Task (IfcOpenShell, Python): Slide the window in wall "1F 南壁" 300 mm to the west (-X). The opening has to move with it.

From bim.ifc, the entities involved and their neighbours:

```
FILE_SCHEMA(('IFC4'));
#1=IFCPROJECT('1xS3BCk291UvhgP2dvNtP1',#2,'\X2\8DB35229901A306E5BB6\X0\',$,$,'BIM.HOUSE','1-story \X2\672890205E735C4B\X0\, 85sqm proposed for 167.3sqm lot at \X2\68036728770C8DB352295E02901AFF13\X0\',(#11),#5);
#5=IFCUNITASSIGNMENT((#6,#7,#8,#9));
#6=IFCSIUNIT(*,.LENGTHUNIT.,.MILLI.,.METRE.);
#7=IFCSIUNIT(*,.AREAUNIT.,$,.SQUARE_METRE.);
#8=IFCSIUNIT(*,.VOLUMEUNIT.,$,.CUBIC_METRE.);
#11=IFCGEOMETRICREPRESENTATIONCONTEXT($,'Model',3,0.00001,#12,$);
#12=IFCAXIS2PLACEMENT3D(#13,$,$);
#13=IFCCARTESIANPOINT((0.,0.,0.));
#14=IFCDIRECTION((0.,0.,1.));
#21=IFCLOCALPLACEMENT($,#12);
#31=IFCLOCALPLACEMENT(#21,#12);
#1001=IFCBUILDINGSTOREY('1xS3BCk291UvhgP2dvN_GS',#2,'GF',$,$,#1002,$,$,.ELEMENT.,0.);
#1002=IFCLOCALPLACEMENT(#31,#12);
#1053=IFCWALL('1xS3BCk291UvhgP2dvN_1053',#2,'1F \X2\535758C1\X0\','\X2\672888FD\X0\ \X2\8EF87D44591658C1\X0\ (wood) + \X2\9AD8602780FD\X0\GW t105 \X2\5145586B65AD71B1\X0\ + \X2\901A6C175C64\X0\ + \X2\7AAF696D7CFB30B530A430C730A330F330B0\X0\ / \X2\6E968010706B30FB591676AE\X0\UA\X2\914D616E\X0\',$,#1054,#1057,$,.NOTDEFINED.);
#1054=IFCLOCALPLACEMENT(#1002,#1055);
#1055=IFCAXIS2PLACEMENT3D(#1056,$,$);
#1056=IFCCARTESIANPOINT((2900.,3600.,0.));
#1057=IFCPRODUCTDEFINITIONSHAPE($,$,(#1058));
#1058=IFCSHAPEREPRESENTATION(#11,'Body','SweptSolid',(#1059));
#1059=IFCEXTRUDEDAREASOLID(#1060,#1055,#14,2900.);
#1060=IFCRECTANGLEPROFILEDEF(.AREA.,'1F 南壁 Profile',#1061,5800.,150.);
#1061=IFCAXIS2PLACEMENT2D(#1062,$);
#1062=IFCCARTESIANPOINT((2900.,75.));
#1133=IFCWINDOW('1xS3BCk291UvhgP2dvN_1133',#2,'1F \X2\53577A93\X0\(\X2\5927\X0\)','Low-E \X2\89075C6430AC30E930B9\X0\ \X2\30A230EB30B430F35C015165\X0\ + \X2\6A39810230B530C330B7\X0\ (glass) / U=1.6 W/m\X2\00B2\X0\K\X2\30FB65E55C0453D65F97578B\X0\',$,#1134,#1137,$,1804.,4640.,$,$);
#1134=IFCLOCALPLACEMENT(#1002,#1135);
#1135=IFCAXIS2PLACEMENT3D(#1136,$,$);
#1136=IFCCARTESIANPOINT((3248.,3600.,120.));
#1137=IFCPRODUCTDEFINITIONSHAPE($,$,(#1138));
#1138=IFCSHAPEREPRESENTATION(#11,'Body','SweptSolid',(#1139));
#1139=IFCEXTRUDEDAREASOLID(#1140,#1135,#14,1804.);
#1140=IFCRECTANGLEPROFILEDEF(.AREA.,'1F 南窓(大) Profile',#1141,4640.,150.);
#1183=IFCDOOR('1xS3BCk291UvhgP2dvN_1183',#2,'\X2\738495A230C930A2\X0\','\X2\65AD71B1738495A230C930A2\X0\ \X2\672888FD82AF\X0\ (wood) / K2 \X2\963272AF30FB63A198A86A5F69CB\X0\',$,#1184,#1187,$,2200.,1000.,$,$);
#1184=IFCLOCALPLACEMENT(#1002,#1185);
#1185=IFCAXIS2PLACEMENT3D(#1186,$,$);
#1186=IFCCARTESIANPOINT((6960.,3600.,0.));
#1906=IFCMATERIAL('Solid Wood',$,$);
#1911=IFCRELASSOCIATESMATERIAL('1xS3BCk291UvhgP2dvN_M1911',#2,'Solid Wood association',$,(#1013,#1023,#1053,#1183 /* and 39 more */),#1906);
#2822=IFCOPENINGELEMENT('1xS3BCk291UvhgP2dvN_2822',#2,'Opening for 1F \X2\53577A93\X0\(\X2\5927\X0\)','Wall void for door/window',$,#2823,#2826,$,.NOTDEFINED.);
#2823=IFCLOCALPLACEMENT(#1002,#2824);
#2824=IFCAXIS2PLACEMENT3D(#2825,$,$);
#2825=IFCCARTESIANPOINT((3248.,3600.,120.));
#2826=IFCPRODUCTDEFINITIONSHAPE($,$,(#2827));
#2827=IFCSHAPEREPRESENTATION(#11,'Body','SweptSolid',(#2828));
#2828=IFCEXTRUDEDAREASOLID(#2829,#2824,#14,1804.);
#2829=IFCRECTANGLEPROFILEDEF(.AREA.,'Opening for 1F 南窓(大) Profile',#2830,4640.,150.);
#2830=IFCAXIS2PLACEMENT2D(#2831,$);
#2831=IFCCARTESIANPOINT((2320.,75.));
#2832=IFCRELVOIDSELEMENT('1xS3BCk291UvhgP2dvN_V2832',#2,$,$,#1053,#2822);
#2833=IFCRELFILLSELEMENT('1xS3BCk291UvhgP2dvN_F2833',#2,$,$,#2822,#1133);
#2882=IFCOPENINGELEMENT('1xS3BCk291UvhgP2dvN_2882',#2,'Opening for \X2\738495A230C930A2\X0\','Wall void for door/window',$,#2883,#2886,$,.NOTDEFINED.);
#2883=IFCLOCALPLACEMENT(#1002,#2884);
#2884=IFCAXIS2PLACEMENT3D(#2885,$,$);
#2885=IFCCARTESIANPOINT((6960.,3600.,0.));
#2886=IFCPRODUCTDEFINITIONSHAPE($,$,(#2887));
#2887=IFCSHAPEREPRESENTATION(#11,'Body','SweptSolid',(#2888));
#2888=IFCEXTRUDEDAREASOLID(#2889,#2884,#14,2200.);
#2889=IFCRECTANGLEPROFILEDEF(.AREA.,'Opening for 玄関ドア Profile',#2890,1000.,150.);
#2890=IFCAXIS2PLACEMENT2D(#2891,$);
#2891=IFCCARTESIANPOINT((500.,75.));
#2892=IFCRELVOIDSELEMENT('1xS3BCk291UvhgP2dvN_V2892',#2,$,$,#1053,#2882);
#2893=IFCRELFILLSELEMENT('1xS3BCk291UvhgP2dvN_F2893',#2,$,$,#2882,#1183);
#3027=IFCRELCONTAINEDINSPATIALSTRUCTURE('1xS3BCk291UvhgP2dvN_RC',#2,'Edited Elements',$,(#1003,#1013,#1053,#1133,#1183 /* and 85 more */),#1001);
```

```python
import ifcopenshell
import ifcopenshell.api.geometry
import ifcopenshell.util.placement
import ifcopenshell.util.unit

model = ifcopenshell.open("bim.ifc")
unit_scale = ifcopenshell.util.unit.calculate_unit_scale(model)

window = model.by_guid("1xS3BCk291UvhgP2dvN_1133")
opening = window.FillsVoids[0].RelatingOpeningElement
wall = opening.VoidsElements[0].RelatingBuildingElement

wall_matrix = ifcopenshell.util.placement.get_local_placement(wall.ObjectPlacement)
shift = wall_matrix[:3, 0] * -0.3 / unit_scale
before = ifcopenshell.util.placement.get_local_placement(window.ObjectPlacement)[:3, 3].copy()

# The window is not placed relative to its opening, so move both.
for product in (opening, window):
    matrix = ifcopenshell.util.placement.get_local_placement(product.ObjectPlacement)
    matrix[:3, 3] += shift
    ifcopenshell.api.geometry.edit_object_placement(model, product=product, matrix=matrix, is_si=False)

after = ifcopenshell.util.placement.get_local_placement(window.ObjectPlacement)[:3, 3]
print("window moved by", (after - before).round(3) + 0.0)

model.write("bim_v2.ifc")
```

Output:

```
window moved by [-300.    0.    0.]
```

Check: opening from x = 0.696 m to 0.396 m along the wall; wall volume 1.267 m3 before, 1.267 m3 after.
